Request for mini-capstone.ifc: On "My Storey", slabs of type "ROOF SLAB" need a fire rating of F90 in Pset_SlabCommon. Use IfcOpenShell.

First a look at what the model holds.

```python
import ifcopenshell
import ifcopenshell.util.element

model = ifcopenshell.open("mini-capstone.ifc")
print(model.schema)
storey = next(s for s in model.by_type("IfcBuildingStorey") if s.Name == "My Storey")
slabs = [e for e in ifcopenshell.util.element.get_decomposition(storey) if e.is_a("IfcSlab")]
seen = {}
for e in slabs:
    element_type = ifcopenshell.util.element.get_type(e)
    key = (element_type.Name if element_type != e and element_type else None, ifcopenshell.util.element.get_pset(e, "Pset_SlabCommon", "FireRating"))
    seen[key] = seen.get(key, 0) + 1
for (name, value), count in sorted(seen.items(), key=str):
    print(count, "x", name, "|", value)
```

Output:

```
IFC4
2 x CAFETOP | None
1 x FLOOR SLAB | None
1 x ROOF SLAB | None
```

```python
import ifcopenshell
import ifcopenshell.api.pset
import ifcopenshell.util.element

model = ifcopenshell.open("mini-capstone.ifc")

storey = next(s for s in model.by_type("IfcBuildingStorey") if s.Name == "My Storey")
slabs = [e for e in ifcopenshell.util.element.get_decomposition(storey) if e.is_a("IfcSlab")]

count = 0
for e in slabs:
    element_type = ifcopenshell.util.element.get_type(e)
    if element_type in (None, e) or element_type.Name != "ROOF SLAB":
        continue
    # add_pset returns the element's existing set when there is one.
    pset = ifcopenshell.api.pset.add_pset(model, product=e, name="Pset_SlabCommon")
    ifcopenshell.api.pset.edit_pset(model, pset=pset, properties={"FireRating": "F90"})
    count += 1

print(count, "slabs updated")

model.write("mini-capstone_updated.ifc")
```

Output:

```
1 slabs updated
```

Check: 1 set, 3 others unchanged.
